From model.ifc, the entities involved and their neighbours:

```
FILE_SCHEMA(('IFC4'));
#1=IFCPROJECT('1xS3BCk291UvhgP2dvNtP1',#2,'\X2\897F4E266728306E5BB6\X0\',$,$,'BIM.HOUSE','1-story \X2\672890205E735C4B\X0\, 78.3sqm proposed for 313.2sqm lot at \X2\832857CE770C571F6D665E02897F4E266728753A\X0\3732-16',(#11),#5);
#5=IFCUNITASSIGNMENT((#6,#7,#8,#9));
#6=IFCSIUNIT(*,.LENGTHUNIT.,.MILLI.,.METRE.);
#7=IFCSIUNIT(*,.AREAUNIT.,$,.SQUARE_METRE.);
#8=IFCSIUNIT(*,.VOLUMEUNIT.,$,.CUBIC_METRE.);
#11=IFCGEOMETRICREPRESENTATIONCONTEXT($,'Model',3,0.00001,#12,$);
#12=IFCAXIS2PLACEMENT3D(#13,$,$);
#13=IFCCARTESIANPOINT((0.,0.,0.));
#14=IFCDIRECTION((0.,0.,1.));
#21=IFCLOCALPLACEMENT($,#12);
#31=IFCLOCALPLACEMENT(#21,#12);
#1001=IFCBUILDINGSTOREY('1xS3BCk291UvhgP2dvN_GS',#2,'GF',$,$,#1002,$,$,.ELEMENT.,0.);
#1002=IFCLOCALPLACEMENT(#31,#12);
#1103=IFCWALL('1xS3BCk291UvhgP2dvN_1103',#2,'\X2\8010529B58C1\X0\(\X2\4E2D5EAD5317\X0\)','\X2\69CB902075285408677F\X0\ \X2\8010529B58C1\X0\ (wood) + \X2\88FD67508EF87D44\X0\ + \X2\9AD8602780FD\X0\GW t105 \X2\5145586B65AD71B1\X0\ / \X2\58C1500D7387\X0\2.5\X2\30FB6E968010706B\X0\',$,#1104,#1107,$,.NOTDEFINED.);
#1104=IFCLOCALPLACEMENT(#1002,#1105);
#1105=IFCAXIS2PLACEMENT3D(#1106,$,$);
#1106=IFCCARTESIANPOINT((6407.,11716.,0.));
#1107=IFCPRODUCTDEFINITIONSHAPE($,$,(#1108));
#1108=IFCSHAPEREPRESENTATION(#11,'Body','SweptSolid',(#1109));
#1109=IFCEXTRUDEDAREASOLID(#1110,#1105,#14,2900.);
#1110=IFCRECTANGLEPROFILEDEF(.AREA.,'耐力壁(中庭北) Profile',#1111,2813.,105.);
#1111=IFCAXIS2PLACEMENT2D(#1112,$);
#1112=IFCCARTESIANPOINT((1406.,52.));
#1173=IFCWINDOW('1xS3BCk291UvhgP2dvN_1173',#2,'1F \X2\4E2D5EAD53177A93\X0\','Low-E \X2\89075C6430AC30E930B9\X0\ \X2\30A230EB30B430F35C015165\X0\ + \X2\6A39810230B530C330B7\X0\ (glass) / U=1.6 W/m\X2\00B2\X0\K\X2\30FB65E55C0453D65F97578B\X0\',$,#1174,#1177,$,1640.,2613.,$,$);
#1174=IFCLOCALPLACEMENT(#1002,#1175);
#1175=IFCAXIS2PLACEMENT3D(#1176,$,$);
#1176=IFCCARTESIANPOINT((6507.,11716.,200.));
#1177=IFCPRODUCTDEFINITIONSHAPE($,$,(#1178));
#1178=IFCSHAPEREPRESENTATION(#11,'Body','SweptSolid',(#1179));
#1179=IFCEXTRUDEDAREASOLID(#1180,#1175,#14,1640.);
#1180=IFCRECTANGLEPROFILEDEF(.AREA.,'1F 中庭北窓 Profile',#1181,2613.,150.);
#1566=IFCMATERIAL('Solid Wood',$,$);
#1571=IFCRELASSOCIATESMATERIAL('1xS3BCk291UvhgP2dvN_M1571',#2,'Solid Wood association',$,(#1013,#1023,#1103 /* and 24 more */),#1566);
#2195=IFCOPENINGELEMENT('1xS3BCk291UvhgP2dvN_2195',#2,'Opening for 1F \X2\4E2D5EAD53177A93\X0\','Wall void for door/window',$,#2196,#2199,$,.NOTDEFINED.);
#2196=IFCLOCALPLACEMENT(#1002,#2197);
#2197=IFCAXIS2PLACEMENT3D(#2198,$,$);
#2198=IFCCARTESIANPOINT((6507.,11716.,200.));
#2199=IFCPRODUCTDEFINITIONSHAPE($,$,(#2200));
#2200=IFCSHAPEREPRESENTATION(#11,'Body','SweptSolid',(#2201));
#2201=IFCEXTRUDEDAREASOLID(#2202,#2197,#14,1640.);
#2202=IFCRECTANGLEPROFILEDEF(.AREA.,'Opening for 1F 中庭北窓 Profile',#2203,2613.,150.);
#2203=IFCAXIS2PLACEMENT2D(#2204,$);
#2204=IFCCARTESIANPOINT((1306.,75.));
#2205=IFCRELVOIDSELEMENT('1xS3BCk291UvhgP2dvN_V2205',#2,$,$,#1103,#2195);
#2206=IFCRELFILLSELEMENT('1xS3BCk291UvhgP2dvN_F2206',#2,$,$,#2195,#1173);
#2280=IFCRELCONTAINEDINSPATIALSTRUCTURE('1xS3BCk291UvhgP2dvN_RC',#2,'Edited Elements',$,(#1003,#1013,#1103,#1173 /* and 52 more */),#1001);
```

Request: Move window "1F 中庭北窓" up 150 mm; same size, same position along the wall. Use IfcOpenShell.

```python
import numpy as np
import ifcopenshell
import ifcopenshell.api.geometry
import ifcopenshell.util.placement
import ifcopenshell.util.unit

model = ifcopenshell.open("model.ifc")
unit_scale = ifcopenshell.util.unit.calculate_unit_scale(model)

window = model.by_id(1173)
opening = window.FillsVoids[0].RelatingOpeningElement
dz = 0.15 / unit_scale

shift = np.array([0.0, 0.0, dz])
# The window is not placed relative to its opening, so move both.
for product in (opening, window):
    matrix = ifcopenshell.util.placement.get_local_placement(product.ObjectPlacement)
    matrix[:3, 3] += shift
    ifcopenshell.api.geometry.edit_object_placement(model, product=product, matrix=matrix, is_si=False)

print(f"moved by {dz * unit_scale:+.3f} m")

model.write("model_edited.ifc")
```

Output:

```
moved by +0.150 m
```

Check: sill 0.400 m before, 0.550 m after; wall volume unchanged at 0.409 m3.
